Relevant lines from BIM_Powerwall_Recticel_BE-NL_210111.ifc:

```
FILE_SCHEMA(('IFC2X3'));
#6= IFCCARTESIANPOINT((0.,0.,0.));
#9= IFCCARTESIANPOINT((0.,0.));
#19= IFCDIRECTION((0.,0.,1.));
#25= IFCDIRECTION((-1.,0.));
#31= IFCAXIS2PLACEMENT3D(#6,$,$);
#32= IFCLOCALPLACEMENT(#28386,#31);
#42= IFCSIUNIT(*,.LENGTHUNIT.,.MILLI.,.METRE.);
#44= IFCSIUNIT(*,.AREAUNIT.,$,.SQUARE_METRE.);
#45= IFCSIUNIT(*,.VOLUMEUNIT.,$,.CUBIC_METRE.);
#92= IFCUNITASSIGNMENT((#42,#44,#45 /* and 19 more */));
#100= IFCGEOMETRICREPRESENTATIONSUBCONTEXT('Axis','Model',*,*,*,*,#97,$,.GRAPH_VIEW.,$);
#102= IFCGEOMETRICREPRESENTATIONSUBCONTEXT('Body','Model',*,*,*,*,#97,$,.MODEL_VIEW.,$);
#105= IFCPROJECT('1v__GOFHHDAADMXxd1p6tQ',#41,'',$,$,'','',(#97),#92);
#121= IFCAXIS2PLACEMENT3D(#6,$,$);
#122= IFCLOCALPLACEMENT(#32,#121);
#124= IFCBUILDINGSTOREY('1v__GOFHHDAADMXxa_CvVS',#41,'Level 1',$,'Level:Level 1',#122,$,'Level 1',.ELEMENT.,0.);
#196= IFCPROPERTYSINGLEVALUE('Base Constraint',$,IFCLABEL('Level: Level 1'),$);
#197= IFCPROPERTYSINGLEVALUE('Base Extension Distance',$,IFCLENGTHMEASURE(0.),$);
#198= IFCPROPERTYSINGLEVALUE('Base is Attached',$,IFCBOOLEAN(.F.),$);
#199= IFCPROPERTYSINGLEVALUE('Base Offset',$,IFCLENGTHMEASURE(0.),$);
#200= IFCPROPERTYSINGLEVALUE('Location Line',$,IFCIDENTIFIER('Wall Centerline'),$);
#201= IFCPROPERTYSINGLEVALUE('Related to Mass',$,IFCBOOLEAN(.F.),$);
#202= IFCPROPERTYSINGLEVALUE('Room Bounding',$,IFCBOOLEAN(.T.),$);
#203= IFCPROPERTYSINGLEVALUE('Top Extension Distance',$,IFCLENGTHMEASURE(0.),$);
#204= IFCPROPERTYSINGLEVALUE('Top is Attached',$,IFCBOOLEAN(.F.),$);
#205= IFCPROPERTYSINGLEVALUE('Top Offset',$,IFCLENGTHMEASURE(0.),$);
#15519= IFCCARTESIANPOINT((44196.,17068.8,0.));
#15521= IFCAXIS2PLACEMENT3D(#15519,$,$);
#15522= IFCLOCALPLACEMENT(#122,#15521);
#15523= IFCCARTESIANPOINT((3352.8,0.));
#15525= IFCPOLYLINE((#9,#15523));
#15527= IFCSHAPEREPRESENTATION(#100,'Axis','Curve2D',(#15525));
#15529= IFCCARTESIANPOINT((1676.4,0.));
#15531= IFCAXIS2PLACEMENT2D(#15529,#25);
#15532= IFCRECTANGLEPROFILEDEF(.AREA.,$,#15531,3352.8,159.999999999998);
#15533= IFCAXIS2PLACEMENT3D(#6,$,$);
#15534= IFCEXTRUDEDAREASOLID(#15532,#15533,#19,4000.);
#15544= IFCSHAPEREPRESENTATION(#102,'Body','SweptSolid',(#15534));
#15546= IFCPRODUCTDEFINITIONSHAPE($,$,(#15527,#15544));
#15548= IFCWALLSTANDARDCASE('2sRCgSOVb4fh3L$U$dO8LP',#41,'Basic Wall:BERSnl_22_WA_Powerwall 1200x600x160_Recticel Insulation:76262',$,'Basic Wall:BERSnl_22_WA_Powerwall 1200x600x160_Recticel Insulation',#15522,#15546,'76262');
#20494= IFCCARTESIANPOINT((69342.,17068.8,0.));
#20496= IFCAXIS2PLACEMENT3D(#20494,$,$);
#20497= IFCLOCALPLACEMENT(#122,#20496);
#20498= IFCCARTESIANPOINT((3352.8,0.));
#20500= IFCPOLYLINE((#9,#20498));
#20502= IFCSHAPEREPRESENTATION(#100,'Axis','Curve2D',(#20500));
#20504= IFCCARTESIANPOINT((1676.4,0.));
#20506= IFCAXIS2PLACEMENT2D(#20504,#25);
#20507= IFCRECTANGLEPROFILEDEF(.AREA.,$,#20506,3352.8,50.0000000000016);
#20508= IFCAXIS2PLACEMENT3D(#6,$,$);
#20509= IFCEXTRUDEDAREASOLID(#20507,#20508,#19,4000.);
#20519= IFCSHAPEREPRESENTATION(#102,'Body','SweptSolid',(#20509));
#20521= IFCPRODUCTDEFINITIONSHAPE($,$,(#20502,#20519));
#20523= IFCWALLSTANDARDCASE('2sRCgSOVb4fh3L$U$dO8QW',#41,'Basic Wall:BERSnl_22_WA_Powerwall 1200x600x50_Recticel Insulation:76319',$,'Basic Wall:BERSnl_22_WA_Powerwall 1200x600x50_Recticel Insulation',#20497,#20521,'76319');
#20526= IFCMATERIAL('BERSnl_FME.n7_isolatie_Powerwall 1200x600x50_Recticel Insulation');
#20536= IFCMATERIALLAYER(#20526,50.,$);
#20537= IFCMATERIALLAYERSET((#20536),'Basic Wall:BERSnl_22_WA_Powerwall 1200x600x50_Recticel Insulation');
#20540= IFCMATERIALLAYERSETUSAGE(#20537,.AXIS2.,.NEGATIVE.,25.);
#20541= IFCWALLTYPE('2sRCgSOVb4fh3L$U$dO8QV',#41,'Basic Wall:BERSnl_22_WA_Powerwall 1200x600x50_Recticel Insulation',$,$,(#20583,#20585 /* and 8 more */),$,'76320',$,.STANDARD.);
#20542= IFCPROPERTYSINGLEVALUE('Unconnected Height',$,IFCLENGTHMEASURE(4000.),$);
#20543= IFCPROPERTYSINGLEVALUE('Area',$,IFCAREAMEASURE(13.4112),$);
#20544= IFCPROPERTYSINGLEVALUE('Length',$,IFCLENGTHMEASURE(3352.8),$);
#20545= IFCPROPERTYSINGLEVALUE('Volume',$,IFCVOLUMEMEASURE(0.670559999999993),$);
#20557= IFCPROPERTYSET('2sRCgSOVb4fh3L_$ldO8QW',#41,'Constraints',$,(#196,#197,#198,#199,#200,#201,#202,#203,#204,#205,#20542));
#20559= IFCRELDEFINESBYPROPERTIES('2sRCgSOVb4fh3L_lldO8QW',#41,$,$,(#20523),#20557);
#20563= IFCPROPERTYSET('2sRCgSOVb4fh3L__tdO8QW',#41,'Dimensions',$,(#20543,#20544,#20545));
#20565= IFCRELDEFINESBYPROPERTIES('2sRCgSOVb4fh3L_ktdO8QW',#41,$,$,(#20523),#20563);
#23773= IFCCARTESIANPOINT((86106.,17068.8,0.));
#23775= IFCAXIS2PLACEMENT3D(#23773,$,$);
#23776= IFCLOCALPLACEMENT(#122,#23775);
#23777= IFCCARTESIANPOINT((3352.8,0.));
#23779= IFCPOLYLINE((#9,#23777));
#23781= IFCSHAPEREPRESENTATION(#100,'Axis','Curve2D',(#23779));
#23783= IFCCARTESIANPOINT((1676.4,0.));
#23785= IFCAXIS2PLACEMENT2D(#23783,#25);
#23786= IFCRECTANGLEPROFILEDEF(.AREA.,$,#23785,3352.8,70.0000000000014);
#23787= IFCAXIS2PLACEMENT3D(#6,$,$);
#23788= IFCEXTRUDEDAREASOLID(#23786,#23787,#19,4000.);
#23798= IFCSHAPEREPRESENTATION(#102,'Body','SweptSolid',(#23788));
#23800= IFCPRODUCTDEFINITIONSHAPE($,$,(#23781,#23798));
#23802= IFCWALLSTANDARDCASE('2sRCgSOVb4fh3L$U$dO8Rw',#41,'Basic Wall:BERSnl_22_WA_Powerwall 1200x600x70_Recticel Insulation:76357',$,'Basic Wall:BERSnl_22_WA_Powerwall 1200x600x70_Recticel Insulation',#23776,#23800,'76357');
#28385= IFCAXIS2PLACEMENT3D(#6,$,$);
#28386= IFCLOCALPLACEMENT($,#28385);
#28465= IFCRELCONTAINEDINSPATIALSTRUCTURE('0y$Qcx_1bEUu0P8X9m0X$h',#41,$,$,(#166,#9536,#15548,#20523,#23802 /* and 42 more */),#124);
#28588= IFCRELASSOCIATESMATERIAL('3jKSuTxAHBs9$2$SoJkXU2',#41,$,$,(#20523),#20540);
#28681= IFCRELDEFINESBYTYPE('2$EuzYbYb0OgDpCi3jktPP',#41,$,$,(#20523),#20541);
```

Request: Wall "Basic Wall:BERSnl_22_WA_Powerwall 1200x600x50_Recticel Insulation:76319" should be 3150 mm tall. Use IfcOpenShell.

```python
import ifcopenshell
import ifcopenshell.api.pset
import ifcopenshell.geom
import ifcopenshell.util.element
import ifcopenshell.util.representation
import ifcopenshell.util.shape
import ifcopenshell.util.unit

model = ifcopenshell.open("BIM_Powerwall_Recticel_BE-NL_210111.ifc")
area_scale = ifcopenshell.util.unit.calculate_unit_scale(model, "AREAUNIT")
volume_scale = ifcopenshell.util.unit.calculate_unit_scale(model, "VOLUMEUNIT")
settings = ifcopenshell.geom.settings()


def volume(element):
    """Net volume in cubic metres, openings subtracted."""
    shape = ifcopenshell.geom.create_shape(settings, element)
    return ifcopenshell.util.shape.get_volume(shape.geometry)


wall = model.by_id(20523)
before = volume(wall)

body = ifcopenshell.util.representation.get_representation(wall, "Model", "Body")
solid = body.Items[0]
old_height = solid.Depth
solid.Depth = 3150.0
after = volume(wall)
thickness = 0.05  # wall thickness in metres

# Update the stored height, areas and volumes.
pset = model.by_id(ifcopenshell.util.element.get_pset(wall, "Constraints", should_inherit=False)["id"])
ifcopenshell.api.pset.edit_pset(model, pset=pset, properties={
    "Unconnected Height": model.create_entity("IfcLengthMeasure", solid.Depth),
})
pset = model.by_id(ifcopenshell.util.element.get_pset(wall, "Dimensions", should_inherit=False)["id"])
ifcopenshell.api.pset.edit_pset(model, pset=pset, properties={
    "Area": model.create_entity("IfcAreaMeasure", after / thickness / area_scale),
    "Volume": model.create_entity("IfcVolumeMeasure", after / volume_scale),
})

print(f"height {old_height:g} -> {solid.Depth:g}, volume {before:.3f} -> {after:.3f} m3")

model.write("BIM_Powerwall_Recticel_BE-NL_210111_updated.ifc")
```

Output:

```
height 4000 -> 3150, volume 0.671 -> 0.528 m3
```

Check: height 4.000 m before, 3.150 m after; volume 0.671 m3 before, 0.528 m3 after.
